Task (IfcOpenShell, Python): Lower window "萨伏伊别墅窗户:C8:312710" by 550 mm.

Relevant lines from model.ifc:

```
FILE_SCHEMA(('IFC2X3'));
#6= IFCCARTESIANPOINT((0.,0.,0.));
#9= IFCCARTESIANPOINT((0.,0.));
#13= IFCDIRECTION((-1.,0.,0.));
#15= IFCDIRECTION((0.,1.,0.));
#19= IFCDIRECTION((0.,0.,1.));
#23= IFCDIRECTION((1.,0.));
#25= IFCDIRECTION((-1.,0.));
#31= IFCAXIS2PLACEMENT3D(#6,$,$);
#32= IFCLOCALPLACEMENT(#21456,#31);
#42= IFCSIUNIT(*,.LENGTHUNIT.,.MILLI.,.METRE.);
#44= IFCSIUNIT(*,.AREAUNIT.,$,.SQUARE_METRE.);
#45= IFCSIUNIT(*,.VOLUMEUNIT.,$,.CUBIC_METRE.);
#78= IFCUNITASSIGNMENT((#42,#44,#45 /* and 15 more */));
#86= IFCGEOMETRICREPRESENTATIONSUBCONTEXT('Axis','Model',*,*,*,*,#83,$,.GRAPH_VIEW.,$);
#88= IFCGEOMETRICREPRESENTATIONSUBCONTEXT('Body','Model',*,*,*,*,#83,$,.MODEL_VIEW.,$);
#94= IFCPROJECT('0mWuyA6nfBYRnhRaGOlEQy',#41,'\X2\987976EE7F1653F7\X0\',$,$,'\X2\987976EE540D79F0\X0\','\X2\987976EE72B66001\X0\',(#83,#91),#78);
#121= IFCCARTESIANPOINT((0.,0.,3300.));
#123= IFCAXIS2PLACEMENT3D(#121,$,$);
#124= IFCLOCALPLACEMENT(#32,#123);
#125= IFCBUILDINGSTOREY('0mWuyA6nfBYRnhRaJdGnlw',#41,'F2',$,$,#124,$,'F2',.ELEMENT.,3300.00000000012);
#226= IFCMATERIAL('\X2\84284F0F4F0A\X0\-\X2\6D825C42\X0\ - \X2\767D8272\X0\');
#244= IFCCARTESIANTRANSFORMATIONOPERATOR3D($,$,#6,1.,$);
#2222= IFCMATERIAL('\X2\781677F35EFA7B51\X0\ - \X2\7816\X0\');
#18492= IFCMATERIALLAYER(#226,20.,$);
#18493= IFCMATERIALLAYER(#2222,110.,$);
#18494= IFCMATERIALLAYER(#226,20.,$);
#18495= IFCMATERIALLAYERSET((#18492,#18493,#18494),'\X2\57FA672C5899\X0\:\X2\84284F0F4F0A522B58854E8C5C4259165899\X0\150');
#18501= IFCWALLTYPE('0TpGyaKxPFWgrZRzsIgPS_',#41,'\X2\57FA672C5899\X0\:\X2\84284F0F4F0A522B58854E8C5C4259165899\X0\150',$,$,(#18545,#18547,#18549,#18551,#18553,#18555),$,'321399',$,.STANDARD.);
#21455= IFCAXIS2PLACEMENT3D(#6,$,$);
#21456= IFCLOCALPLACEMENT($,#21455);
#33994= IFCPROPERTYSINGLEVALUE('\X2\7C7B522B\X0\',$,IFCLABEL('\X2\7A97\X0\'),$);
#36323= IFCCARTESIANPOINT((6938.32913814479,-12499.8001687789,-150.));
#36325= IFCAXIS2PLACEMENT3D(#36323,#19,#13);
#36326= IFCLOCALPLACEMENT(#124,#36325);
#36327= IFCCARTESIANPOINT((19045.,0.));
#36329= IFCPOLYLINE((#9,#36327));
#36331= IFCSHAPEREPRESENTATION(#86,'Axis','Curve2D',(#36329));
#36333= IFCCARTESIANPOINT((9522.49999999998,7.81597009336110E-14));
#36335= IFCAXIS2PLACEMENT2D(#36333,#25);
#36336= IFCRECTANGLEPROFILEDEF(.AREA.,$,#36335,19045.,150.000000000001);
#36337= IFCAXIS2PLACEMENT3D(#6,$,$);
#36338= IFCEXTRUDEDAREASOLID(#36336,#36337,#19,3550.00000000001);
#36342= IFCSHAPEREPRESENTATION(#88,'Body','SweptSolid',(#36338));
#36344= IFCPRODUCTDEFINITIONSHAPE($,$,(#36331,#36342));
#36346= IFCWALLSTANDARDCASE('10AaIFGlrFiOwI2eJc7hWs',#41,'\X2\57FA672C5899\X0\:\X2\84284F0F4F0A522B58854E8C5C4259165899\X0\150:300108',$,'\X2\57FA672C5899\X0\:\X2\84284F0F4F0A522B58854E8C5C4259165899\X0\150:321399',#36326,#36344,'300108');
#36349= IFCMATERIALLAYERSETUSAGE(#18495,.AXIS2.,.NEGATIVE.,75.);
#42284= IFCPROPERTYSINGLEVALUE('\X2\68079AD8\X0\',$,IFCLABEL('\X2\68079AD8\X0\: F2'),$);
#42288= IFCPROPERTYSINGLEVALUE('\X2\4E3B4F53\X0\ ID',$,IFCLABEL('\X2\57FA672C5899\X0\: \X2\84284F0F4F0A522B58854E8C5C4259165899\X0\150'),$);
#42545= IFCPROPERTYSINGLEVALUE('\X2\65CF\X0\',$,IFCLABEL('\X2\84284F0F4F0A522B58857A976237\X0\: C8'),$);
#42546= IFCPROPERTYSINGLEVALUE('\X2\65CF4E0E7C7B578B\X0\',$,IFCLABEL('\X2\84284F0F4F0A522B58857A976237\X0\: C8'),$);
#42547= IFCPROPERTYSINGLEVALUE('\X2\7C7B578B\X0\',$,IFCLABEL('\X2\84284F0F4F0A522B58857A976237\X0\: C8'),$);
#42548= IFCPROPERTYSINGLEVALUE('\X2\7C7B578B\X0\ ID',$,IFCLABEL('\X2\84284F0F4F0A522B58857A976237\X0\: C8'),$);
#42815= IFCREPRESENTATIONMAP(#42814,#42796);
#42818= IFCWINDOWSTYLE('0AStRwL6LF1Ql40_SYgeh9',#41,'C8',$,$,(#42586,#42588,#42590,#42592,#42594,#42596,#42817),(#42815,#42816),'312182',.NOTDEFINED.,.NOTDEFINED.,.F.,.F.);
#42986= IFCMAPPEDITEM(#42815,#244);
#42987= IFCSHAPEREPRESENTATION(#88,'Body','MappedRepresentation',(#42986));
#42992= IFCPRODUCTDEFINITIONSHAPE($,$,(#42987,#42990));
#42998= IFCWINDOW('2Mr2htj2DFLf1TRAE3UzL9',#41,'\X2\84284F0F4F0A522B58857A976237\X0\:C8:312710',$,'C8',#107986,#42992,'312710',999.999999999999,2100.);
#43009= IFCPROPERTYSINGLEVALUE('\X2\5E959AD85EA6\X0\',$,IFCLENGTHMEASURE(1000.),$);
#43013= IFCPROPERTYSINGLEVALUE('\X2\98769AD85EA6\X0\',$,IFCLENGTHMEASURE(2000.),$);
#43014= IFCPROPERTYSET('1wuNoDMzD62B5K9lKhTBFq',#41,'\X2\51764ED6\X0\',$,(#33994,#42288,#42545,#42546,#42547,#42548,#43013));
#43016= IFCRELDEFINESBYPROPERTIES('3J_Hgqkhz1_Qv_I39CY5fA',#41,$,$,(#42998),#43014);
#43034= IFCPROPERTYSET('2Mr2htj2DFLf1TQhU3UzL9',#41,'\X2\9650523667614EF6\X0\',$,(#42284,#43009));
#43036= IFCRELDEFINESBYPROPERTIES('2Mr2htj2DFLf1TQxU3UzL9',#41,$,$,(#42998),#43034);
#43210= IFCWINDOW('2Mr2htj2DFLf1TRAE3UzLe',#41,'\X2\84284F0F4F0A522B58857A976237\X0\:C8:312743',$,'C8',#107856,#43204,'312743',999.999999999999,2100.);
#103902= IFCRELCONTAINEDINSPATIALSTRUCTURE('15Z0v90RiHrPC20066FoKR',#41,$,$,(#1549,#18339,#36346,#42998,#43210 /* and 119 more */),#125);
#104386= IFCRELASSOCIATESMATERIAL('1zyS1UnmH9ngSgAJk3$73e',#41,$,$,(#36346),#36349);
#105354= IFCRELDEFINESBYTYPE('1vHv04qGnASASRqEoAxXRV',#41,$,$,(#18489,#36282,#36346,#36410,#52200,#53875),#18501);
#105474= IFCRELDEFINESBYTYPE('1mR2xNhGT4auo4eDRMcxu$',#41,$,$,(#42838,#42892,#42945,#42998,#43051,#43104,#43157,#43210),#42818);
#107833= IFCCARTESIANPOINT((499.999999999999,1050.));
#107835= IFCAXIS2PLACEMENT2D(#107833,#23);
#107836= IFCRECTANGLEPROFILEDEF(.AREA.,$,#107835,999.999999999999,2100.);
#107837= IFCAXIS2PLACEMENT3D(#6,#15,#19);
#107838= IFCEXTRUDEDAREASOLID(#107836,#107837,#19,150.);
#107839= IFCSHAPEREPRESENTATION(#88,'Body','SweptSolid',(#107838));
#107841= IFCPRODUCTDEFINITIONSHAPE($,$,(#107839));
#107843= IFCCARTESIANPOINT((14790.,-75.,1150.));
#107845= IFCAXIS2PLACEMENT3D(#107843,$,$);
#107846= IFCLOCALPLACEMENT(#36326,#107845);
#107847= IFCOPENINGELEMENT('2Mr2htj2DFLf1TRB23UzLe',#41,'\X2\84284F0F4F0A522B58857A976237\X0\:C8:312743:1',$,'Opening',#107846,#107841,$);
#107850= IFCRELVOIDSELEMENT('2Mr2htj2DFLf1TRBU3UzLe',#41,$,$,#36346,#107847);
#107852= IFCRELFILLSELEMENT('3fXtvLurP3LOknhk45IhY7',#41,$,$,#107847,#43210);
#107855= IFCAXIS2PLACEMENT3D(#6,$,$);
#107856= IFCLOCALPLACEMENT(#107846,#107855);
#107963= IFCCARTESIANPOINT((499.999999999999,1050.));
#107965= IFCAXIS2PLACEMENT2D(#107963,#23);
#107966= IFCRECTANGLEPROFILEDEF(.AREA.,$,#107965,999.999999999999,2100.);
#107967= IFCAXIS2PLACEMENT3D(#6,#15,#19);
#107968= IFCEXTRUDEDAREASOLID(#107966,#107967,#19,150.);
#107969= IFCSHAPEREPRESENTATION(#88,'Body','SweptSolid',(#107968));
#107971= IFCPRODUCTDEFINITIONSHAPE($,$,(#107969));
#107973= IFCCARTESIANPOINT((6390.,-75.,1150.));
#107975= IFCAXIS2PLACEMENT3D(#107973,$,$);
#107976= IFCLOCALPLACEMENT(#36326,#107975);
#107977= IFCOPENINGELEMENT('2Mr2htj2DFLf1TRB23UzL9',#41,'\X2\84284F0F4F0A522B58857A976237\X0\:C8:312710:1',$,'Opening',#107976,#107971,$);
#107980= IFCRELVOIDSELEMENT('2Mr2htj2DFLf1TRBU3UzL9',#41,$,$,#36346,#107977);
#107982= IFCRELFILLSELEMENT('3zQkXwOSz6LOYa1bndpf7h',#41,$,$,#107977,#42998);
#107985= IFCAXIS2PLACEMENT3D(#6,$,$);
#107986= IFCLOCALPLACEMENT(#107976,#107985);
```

```python
import numpy as np
import ifcopenshell
import ifcopenshell.api.geometry
import ifcopenshell.api.pset
import ifcopenshell.util.element
import ifcopenshell.util.placement
import ifcopenshell.util.unit

model = ifcopenshell.open("model.ifc")
unit_scale = ifcopenshell.util.unit.calculate_unit_scale(model)

window = model.by_guid("2Mr2htj2DFLf1TRAE3UzL9")
opening = window.FillsVoids[0].RelatingOpeningElement
dz = -550.0

shift = np.array([0.0, 0.0, dz])
# The window is placed relative to its opening, so it follows when the opening moves.
matrix = ifcopenshell.util.placement.get_local_placement(opening.ObjectPlacement)
matrix[:3, 3] += shift
ifcopenshell.api.geometry.edit_object_placement(
    model, product=opening, matrix=matrix, is_si=False, should_transform_children=True
)

# Keep the stored heights in step.
pset = model.by_id(ifcopenshell.util.element.get_pset(window, "其他", should_inherit=False)["id"])
ifcopenshell.api.pset.edit_pset(model, pset=pset, properties={
    "顶高度": model.create_entity("IfcLengthMeasure", ifcopenshell.util.element.get_pset(window, "其他", "顶高度") + dz),
})
pset = model.by_id(ifcopenshell.util.element.get_pset(window, "限制条件", should_inherit=False)["id"])
ifcopenshell.api.pset.edit_pset(model, pset=pset, properties={
    "底高度": model.create_entity("IfcLengthMeasure", ifcopenshell.util.element.get_pset(window, "限制条件", "底高度") + dz),
})

print(f"moved by {dz * unit_scale:+.3f} m")

model.write("model_v2.ifc")
```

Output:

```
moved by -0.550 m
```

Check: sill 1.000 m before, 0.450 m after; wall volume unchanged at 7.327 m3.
